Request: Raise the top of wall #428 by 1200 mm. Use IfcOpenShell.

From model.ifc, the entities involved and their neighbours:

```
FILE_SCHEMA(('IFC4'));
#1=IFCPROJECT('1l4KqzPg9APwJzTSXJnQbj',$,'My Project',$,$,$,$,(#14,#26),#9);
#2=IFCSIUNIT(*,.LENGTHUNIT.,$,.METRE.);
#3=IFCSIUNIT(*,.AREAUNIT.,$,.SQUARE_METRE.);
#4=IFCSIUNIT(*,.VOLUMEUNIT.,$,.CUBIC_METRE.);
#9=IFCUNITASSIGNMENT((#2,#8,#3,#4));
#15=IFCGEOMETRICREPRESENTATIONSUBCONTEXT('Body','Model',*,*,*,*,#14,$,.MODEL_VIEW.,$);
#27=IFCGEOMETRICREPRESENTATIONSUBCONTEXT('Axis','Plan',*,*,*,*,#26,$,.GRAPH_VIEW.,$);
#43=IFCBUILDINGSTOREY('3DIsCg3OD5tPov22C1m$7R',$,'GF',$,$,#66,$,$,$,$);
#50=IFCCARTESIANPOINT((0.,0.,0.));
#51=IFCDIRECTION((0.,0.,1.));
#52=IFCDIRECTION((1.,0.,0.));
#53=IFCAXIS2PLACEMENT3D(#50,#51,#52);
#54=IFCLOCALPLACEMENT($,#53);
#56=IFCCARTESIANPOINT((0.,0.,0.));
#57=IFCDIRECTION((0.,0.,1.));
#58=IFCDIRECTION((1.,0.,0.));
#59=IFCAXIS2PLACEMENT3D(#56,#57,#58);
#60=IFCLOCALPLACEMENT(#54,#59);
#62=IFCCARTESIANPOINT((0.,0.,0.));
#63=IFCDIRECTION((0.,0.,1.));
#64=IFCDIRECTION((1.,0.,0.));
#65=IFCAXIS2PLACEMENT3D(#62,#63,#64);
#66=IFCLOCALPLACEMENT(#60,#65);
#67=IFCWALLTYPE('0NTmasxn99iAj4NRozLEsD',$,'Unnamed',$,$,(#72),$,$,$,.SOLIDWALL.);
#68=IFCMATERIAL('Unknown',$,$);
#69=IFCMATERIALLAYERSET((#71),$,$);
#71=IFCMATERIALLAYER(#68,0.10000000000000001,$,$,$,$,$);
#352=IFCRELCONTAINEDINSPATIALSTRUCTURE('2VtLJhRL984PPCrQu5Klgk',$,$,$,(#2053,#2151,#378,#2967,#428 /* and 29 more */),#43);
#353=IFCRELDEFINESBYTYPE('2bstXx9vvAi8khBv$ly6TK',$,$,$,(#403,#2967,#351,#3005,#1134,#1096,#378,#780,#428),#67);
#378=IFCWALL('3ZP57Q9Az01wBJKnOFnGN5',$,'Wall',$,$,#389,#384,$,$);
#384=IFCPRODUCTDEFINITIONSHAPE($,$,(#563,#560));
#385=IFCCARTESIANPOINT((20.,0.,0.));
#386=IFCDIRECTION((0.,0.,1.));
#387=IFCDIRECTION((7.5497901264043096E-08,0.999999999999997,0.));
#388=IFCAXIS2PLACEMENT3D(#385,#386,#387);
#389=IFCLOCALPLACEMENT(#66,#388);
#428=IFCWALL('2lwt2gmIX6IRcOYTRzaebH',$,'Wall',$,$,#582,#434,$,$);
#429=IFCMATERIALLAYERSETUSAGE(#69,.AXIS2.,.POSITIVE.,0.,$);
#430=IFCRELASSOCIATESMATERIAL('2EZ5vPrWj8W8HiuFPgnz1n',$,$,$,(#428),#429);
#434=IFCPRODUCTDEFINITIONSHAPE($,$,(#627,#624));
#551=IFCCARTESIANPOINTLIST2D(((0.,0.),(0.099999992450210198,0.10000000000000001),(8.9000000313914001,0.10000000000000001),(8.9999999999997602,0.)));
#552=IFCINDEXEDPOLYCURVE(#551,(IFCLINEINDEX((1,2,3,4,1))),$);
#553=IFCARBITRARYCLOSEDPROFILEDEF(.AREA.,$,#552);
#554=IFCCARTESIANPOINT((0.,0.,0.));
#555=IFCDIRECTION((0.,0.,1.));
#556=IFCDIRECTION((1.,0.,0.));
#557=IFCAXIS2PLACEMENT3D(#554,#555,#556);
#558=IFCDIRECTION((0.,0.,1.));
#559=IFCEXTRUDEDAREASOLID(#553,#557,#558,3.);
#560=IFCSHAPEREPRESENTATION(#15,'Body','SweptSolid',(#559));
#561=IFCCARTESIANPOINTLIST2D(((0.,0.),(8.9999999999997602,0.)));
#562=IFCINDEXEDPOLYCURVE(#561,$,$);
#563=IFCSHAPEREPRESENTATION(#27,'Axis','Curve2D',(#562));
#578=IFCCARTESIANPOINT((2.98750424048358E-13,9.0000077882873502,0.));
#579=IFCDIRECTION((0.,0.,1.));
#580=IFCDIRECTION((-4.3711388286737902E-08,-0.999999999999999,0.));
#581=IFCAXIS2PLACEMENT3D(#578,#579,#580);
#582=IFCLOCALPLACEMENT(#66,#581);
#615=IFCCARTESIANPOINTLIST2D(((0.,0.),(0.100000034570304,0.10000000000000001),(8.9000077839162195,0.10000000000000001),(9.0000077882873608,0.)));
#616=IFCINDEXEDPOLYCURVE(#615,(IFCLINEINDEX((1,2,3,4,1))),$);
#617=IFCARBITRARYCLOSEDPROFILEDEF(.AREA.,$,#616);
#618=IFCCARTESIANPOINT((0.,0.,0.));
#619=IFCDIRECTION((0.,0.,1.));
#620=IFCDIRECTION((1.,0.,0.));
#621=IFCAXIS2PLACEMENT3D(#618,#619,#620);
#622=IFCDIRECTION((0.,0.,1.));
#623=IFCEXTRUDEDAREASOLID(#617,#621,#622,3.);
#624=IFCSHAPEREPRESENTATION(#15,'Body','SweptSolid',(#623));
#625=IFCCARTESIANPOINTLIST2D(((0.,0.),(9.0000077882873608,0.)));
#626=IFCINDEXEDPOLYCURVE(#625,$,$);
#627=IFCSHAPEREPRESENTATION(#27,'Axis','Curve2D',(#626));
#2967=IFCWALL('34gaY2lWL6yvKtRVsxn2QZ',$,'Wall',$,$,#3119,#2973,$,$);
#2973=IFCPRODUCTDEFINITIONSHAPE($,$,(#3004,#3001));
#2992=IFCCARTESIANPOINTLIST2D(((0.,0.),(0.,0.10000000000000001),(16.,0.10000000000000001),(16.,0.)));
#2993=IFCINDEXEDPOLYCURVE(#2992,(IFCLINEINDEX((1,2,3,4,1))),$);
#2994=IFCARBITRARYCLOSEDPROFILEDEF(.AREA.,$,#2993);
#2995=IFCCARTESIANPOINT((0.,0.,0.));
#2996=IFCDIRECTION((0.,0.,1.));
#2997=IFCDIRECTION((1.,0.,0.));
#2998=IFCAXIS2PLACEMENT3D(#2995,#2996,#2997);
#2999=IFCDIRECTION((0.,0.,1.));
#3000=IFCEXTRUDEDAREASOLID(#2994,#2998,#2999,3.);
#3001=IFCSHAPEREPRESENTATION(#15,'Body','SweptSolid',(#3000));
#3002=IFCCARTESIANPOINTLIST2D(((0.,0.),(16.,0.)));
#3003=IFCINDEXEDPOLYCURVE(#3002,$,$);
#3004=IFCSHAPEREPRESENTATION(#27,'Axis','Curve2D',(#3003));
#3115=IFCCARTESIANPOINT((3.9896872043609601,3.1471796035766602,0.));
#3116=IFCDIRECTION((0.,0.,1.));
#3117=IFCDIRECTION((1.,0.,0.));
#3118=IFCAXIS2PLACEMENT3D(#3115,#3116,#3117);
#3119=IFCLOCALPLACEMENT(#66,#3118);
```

```python
import ifcopenshell
import ifcopenshell.geom
import ifcopenshell.util.representation
import ifcopenshell.util.shape

model = ifcopenshell.open("model.ifc")
settings = ifcopenshell.geom.settings()


def volume(element):
    """Net volume in cubic metres, openings subtracted."""
    shape = ifcopenshell.geom.create_shape(settings, element)
    return ifcopenshell.util.shape.get_volume(shape.geometry)


wall = model.by_guid("2lwt2gmIX6IRcOYTRzaebH")
before = volume(wall)

body = ifcopenshell.util.representation.get_representation(wall, "Model", "Body")
solid = body.Items[0]
old_height = solid.Depth
solid.Depth += 1.2
after = volume(wall)

print(f"height {old_height:g} -> {solid.Depth:g}, volume {before:.3f} -> {after:.3f} m3")

model.write("model_v2.ifc")
```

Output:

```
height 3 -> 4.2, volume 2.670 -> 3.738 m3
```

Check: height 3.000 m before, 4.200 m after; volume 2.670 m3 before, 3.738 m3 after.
